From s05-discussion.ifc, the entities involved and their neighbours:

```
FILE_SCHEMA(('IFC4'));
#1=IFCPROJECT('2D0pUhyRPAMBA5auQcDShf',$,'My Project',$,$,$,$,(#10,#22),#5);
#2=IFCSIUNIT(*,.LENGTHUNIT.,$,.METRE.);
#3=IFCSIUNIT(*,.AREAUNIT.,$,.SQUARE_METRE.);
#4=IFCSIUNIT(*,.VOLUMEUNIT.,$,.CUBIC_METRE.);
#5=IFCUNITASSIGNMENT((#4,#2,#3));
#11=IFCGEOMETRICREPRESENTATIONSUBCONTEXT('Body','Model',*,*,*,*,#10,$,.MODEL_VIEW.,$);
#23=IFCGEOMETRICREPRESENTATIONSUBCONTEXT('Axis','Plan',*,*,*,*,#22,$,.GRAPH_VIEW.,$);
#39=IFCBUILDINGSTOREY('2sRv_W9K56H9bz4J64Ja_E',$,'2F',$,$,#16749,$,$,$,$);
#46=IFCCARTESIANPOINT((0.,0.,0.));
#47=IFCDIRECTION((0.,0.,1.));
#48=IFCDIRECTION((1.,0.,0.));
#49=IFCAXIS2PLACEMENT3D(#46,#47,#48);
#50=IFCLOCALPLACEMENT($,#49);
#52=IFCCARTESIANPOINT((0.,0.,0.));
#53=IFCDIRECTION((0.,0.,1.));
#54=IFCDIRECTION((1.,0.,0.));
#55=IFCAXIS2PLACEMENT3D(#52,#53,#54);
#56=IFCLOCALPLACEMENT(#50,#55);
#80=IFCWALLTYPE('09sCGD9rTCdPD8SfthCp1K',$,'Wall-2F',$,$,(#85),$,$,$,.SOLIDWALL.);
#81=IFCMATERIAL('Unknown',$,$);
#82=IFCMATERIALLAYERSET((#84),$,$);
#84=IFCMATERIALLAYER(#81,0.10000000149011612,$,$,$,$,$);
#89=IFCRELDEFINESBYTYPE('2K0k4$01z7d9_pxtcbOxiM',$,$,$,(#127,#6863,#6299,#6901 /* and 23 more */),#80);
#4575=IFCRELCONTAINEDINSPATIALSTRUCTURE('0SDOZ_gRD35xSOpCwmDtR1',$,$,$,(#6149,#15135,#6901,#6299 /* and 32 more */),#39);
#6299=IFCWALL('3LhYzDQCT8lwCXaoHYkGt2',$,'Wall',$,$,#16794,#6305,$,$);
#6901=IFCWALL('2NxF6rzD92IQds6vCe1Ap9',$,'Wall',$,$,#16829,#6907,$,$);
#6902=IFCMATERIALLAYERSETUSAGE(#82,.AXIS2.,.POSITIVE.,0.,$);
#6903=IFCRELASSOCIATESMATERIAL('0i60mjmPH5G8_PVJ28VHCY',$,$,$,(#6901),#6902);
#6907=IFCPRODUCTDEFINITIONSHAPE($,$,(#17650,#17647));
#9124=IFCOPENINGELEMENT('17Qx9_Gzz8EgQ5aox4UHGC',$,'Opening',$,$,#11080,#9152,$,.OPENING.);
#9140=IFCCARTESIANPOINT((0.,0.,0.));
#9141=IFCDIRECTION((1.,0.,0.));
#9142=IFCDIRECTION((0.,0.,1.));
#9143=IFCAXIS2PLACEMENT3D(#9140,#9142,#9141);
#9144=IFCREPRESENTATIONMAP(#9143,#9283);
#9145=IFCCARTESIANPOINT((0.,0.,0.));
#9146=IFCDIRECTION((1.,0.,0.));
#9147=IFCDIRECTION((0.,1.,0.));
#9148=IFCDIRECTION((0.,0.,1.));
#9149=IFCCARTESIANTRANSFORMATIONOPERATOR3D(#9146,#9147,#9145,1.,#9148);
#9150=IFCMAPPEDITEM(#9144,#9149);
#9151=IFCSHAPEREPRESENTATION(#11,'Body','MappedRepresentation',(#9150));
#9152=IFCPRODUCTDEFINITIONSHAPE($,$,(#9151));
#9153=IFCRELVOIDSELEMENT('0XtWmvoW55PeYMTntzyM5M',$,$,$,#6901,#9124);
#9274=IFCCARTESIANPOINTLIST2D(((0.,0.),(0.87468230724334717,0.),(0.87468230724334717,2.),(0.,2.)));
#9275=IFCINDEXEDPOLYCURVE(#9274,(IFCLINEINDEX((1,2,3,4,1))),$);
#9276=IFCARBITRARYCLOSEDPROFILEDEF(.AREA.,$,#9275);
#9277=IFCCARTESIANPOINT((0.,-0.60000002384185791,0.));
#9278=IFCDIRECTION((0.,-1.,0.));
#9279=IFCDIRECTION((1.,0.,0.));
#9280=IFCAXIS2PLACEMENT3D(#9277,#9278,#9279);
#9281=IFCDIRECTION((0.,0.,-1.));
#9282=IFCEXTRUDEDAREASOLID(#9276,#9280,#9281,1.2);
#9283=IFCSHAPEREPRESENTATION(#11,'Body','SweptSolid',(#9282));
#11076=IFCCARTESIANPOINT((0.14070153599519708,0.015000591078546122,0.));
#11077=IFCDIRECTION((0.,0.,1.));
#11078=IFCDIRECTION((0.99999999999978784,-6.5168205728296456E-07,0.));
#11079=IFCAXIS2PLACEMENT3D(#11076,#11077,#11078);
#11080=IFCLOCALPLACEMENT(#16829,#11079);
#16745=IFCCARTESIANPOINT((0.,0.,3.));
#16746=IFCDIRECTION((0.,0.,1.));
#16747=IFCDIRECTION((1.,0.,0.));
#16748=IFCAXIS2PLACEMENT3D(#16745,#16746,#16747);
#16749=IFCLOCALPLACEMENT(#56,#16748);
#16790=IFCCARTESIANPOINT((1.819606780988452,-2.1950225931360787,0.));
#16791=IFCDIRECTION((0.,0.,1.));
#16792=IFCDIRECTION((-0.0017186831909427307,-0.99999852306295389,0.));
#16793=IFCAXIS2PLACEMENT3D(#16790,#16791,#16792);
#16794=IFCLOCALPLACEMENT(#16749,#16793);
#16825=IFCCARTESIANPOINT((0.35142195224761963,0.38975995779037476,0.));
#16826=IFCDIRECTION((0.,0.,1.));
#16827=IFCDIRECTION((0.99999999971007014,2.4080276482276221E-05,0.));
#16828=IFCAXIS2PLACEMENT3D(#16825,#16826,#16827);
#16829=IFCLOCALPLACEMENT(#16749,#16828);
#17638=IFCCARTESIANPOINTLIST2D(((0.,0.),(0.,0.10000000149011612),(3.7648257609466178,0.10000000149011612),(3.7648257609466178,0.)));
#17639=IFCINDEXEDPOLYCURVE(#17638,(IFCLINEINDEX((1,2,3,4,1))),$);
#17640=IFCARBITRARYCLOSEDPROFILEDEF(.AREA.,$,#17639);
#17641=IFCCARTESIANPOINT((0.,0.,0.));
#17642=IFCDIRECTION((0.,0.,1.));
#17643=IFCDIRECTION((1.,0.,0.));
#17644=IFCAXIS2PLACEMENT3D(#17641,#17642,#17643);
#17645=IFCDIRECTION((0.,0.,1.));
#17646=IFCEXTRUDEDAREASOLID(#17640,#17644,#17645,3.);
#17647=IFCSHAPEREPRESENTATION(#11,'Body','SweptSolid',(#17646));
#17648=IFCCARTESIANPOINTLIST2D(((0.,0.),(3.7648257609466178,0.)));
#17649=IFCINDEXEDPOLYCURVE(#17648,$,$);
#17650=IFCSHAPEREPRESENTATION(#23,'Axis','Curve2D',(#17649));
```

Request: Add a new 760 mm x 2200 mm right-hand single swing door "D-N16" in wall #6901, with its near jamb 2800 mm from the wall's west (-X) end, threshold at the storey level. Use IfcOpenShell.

```python
import numpy as np
import ifcopenshell
import ifcopenshell.api.feature
import ifcopenshell.api.geometry
import ifcopenshell.api.root
import ifcopenshell.api.spatial
import ifcopenshell.geom
import ifcopenshell.util.element
import ifcopenshell.util.placement
import ifcopenshell.util.representation
import ifcopenshell.util.shape
import ifcopenshell.util.unit

model = ifcopenshell.open("s05-discussion.ifc")
unit_scale = ifcopenshell.util.unit.calculate_unit_scale(model)
settings = ifcopenshell.geom.settings()


def volume(element):
    """Net volume in cubic metres, openings subtracted."""
    shape = ifcopenshell.geom.create_shape(settings, element)
    return ifcopenshell.util.shape.get_volume(shape.geometry)


wall = model.by_id(6901)
storey = ifcopenshell.util.element.get_container(wall, ifc_class="IfcBuildingStorey")
context = ifcopenshell.util.representation.get_context(model, "Model", "Body", "MODEL_VIEW")
before = volume(wall)

width, height, from_end, sill = 0.76, 2.2, 2.8, 0.0  # metres

# The wall runs along its own X axis, and the end named is its -X end.
wall_shape = ifcopenshell.geom.create_shape(settings, wall)
x, y, z = ifcopenshell.util.shape.get_vertices(wall_shape.geometry).T
start = x.min() + from_end
face, thickness = float(y.min()), float(y.max() - y.min())
wall_matrix = ifcopenshell.util.placement.get_local_placement(wall.ObjectPlacement)
level = ifcopenshell.util.placement.get_local_placement(storey.ObjectPlacement)[2, 3]


def in_wall(x, y):
    """Placement at x, y metres in the wall's axes, at sill height."""
    matrix = wall_matrix.copy()
    matrix[:, 3] = wall_matrix @ np.array([x / unit_scale, y / unit_scale, 0.0, 1.0])
    matrix[2, 3] = level + sill / unit_scale
    return matrix


# Opening: a box that overshoots both wall faces by 50 mm.
opening = ifcopenshell.api.root.create_entity(model, ifc_class="IfcOpeningElement", predefined_type="OPENING")
box = ifcopenshell.api.geometry.add_wall_representation(
    model, context=context, length=width, height=height, thickness=thickness + 0.1
)
ifcopenshell.api.geometry.assign_representation(model, product=opening, representation=box)
ifcopenshell.api.geometry.edit_object_placement(model, product=opening, matrix=in_wall(start, face - 0.05), is_si=False)
ifcopenshell.api.feature.add_feature(model, feature=opening, element=wall)

door = ifcopenshell.api.root.create_entity(model, ifc_class="IfcDoor", name="D-N16", predefined_type="DOOR")
door.OverallWidth, door.OverallHeight = width / unit_scale, height / unit_scale
door.OperationType = "SINGLE_SWING_RIGHT"
body = ifcopenshell.api.geometry.add_door_representation(
    model,
    context=context,
    overall_width=door.OverallWidth,
    overall_height=door.OverallHeight,
    operation_type="SINGLE_SWING_RIGHT",
    lining_properties={"LiningDepth": thickness / unit_scale, "ThresholdDepth": thickness / unit_scale},
)
ifcopenshell.api.geometry.assign_representation(model, product=door, representation=body)
ifcopenshell.api.spatial.assign_container(model, products=[door], relating_structure=storey)
ifcopenshell.api.feature.add_filling(model, opening=opening, element=door)

# The lining spans the wall, so the door starts at the wall face.
ifcopenshell.api.geometry.edit_object_placement(model, product=door, matrix=in_wall(start, face), is_si=False)

after = volume(wall)

print(f"wall volume {before:.3f} -> {after:.3f} m3")

model.write("s05-discussion_updated.ifc")
```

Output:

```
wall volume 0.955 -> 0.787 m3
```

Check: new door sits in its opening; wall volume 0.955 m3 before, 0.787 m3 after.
